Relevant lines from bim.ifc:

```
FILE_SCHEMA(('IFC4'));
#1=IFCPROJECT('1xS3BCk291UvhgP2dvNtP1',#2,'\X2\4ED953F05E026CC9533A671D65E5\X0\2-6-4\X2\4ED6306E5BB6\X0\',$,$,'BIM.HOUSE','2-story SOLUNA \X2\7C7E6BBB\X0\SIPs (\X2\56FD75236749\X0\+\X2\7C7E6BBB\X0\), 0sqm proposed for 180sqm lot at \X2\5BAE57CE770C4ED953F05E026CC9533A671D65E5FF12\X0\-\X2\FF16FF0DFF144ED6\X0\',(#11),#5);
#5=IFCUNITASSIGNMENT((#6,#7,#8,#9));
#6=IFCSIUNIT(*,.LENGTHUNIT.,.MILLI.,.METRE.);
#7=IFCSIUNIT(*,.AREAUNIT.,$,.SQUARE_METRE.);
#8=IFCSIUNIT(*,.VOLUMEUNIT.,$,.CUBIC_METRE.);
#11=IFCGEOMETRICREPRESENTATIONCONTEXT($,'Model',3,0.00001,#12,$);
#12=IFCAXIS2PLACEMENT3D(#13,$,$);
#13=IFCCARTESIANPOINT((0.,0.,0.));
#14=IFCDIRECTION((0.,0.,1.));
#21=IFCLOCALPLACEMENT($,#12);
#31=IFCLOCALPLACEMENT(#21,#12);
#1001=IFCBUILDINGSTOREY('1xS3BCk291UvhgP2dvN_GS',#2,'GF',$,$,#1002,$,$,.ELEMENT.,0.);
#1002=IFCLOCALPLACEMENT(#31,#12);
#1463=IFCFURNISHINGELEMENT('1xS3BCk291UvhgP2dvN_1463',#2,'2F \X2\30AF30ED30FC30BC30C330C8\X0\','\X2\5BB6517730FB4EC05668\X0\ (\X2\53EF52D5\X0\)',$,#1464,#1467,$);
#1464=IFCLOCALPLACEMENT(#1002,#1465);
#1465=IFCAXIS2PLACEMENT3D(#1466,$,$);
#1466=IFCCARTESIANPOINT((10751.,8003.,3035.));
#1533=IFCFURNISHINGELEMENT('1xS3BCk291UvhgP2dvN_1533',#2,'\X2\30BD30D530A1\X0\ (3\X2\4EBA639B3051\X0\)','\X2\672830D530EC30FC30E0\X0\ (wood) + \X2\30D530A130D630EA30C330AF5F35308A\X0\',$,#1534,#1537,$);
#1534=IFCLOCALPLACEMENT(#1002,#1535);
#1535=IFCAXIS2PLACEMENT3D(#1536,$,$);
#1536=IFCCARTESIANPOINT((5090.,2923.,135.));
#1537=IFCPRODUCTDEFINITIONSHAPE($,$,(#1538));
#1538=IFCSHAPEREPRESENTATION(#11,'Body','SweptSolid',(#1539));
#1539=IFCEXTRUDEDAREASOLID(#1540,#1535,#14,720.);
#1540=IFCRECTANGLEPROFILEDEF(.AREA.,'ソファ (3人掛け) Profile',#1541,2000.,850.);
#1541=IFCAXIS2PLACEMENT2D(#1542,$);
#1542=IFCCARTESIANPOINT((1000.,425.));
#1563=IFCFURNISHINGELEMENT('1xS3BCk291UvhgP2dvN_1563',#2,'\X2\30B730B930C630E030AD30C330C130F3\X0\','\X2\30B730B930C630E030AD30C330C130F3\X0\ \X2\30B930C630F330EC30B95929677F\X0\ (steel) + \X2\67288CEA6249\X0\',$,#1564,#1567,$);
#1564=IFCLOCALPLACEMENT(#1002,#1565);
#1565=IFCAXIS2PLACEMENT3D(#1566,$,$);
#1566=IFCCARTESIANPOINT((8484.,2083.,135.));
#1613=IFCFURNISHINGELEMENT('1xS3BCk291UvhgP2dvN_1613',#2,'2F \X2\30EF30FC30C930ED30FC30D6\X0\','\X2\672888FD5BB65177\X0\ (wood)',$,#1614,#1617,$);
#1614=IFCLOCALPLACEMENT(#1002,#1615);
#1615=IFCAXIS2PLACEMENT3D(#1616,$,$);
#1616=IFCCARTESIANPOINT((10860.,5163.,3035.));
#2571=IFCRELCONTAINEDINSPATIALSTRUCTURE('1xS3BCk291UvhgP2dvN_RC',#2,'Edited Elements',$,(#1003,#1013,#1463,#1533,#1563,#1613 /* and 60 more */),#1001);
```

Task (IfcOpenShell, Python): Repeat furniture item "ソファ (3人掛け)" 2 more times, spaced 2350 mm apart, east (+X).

```python
import numpy as np
import ifcopenshell
import ifcopenshell.api.geometry
import ifcopenshell.api.root
import ifcopenshell.util.element
import ifcopenshell.util.placement
import ifcopenshell.util.unit

model = ifcopenshell.open("bim.ifc")
unit_scale = ifcopenshell.util.unit.calculate_unit_scale(model)


def reuse_history(source, copy):
    """copy_class also copies each property set's owner history, people and application; keep the originals."""
    for rel in copy.IsDefinedBy:
        if rel.is_a("IfcRelDefinesByProperties") and (history := rel.RelatingPropertyDefinition.OwnerHistory):
            rel.RelatingPropertyDefinition.OwnerHistory = source.OwnerHistory
            ifcopenshell.util.element.remove_deep2(model, history)


source = model.by_id(1533)
base = ifcopenshell.util.placement.get_local_placement(source.ObjectPlacement)
step = np.array([1.0, 0.0, 0.0]) * 2.35 / unit_scale

for i in range(1, 3):
    copy = ifcopenshell.api.root.copy_class(model, product=source)
    copy.Representation = ifcopenshell.util.element.copy_deep(
        model, source.Representation, exclude=["IfcGeometricRepresentationContext", "IfcRepresentationMap"]
    )
    reuse_history(source, copy)
    matrix = base.copy()
    matrix[:3, 3] += i * step
    print("added at", matrix[:3, 3].round(3) + 0.0)
    ifcopenshell.api.geometry.edit_object_placement(model, product=copy, matrix=matrix, is_si=False)

model.write("bim-out.ifc")
```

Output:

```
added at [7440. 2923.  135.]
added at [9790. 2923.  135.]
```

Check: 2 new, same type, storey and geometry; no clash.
